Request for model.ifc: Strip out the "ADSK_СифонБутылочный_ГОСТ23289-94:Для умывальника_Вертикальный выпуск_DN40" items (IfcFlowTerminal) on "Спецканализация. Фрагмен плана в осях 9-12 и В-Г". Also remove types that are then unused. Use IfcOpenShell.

First a look at what the model holds.

```python
import ifcopenshell
import ifcopenshell.util.element

model = ifcopenshell.open("model.ifc")
print(model.schema)
storey = next(s for s in model.by_type("IfcBuildingStorey") if s.Name == "Спецканализация. Фрагмен плана в осях 9-12 и В-Г")
terminals = [e for e in ifcopenshell.util.element.get_decomposition(storey) if e.is_a("IfcFlowTerminal")]
seen = {}
for e in terminals:
    element_type = ifcopenshell.util.element.get_type(e)
    name = element_type.Name if element_type not in (None, e) else None
    seen[name] = seen.get(name, 0) + 1
for name, count in sorted(seen.items(), key=str):
    print(count, "x", name)
```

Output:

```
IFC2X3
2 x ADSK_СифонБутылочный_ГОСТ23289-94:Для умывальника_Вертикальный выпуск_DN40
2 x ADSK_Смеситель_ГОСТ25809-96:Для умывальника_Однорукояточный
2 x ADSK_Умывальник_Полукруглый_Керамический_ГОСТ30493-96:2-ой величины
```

```python
import ifcopenshell
import ifcopenshell.api.root
import ifcopenshell.util.element

model = ifcopenshell.open("model.ifc")

storey = next(s for s in model.by_type("IfcBuildingStorey") if s.Name == "Спецканализация. Фрагмен плана в осях 9-12 и В-Г")
terminals = [e for e in ifcopenshell.util.element.get_decomposition(storey) if e.is_a("IfcFlowTerminal")]
targets = [e for e in terminals if (t := ifcopenshell.util.element.get_type(e)) not in (None, e) and t.Name == "ADSK_СифонБутылочный_ГОСТ23289-94:Для умывальника_Вертикальный выпуск_DN40"]
types = {ifcopenshell.util.element.get_type(e) for e in targets} - {None, *targets}

for e in targets:
    ifcopenshell.api.root.remove_product(model, product=e)
print(len(targets), "removed")

unused = [t for t in types if not ifcopenshell.util.element.get_types(t)]
for t in unused:
    ifcopenshell.api.root.remove_product(model, product=t)
print(len(unused), "unused types removed")

model.write("model-out.ifc")
```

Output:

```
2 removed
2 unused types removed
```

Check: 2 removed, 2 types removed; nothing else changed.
